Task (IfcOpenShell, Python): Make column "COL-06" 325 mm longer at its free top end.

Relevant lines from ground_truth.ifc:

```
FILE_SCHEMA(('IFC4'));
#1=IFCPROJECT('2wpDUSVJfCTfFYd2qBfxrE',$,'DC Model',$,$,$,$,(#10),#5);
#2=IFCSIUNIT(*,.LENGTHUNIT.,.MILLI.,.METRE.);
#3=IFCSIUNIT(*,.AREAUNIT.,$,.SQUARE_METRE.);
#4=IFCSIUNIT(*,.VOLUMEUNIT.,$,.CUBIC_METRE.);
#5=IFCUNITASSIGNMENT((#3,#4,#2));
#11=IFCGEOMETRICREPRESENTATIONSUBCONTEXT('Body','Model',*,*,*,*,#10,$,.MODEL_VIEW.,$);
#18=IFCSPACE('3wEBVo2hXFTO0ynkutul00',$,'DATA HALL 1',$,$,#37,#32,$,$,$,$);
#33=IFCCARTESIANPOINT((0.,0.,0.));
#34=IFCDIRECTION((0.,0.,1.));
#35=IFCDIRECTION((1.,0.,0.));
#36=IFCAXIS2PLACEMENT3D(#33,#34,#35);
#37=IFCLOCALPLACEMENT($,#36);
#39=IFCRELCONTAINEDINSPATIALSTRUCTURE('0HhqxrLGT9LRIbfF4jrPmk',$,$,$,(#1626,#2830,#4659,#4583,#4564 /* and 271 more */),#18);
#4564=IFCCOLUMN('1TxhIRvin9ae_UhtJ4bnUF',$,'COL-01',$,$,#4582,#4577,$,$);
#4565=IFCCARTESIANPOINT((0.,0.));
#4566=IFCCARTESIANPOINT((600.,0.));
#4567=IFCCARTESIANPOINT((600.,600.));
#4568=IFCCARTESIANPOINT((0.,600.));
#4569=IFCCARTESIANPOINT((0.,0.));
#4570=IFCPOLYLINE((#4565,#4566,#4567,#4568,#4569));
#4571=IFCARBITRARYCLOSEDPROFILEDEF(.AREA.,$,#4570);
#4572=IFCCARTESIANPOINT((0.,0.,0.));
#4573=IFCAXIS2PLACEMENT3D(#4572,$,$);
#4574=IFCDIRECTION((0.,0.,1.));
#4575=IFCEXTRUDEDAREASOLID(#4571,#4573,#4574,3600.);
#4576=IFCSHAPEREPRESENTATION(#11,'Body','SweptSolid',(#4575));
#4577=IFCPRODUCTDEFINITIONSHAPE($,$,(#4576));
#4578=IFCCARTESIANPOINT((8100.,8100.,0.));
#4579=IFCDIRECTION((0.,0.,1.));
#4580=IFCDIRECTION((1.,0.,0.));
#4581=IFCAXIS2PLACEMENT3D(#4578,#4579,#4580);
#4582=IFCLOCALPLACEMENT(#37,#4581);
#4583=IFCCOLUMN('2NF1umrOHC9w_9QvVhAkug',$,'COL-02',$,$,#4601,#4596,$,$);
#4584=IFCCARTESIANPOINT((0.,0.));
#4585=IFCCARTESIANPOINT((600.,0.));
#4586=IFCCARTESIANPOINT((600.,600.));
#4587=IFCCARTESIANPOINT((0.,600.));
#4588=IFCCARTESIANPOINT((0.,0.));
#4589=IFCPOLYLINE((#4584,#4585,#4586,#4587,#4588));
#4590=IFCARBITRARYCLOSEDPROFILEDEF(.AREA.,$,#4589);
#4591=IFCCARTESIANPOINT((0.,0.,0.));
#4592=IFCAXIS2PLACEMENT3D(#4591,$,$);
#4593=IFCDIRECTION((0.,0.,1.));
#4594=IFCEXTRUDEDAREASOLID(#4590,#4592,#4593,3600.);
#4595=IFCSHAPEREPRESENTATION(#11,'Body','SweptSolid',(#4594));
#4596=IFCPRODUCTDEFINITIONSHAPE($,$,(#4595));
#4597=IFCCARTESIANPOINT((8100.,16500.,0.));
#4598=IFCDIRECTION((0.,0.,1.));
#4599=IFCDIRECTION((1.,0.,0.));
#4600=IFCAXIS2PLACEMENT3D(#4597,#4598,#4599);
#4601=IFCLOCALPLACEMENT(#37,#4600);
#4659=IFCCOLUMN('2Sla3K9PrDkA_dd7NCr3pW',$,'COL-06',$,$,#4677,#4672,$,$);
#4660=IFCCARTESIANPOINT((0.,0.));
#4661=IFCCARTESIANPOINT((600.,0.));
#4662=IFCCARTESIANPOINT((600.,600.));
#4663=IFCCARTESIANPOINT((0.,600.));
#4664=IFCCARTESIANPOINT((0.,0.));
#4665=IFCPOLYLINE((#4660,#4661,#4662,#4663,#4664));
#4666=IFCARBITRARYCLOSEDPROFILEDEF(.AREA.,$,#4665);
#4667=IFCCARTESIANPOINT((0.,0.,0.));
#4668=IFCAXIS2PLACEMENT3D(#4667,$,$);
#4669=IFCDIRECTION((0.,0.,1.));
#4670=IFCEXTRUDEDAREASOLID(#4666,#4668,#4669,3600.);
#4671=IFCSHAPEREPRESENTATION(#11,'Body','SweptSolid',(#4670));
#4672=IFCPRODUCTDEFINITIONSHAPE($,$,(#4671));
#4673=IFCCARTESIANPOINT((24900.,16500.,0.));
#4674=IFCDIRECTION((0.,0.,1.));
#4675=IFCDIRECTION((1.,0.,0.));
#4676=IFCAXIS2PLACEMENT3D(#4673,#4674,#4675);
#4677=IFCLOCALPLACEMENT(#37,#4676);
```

```python
import ifcopenshell
import ifcopenshell.util.representation

model = ifcopenshell.open("ground_truth.ifc")

member = model.by_guid("2Sla3K9PrDkA_dd7NCr3pW")
change = 325.0

# The extrusion runs towards the end named, so only its depth changes.
body = ifcopenshell.util.representation.get_representation(member, "Model", "Body")
solid = body.Items[0]
old_length = solid.Depth
solid.Depth += change

print(f"length {old_length:g} -> {solid.Depth:g}")

model.write("ground_truth_v2.ifc")
```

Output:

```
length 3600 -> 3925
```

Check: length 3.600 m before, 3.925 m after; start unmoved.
